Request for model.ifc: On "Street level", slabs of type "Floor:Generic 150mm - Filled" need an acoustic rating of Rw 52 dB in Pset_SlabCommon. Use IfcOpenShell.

First a look at what the model holds.

```python
import ifcopenshell
import ifcopenshell.util.element

model = ifcopenshell.open("model.ifc")
print(model.schema)
storey = next(s for s in model.by_type("IfcBuildingStorey") if s.Name == "Street level")
slabs = [e for e in ifcopenshell.util.element.get_decomposition(storey) if e.is_a("IfcSlab")]
seen = {}
for e in slabs:
    element_type = ifcopenshell.util.element.get_type(e)
    key = (element_type.Name if element_type != e and element_type else None, ifcopenshell.util.element.get_pset(e, "Pset_SlabCommon", "AcousticRating"))
    seen[key] = seen.get(key, 0) + 1
for (name, value), count in sorted(seen.items(), key=str):
    print(count, "x", name, "|", value)
```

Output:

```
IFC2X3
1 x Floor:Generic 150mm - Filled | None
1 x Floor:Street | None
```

```python
import ifcopenshell
import ifcopenshell.api.pset
import ifcopenshell.util.element

model = ifcopenshell.open("model.ifc")

storey = next(s for s in model.by_type("IfcBuildingStorey") if s.Name == "Street level")
slabs = [e for e in ifcopenshell.util.element.get_decomposition(storey) if e.is_a("IfcSlab")]

count = 0
for e in slabs:
    element_type = ifcopenshell.util.element.get_type(e)
    if element_type in (None, e) or element_type.Name != "Floor:Generic 150mm - Filled":
        continue
    # add_pset returns the element's existing set when there is one.
    pset = ifcopenshell.api.pset.add_pset(model, product=e, name="Pset_SlabCommon")
    ifcopenshell.api.pset.edit_pset(model, pset=pset, properties={"AcousticRating": "Rw 52 dB"})
    count += 1

print(count, "slabs updated")

model.write("model-out.ifc")
```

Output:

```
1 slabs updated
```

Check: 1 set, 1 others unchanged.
